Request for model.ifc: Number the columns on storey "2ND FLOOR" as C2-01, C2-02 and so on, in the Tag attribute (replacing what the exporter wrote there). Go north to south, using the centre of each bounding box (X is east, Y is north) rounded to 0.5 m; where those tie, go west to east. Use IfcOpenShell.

First a look at what the model holds.

```python
import ifcopenshell
import ifcopenshell.util.element
import ifcopenshell.util.placement

model = ifcopenshell.open("model.ifc")
print(model.schema)
storey = next(s for s in model.by_type("IfcBuildingStorey") if s.Name == "2ND FLOOR")
columns = [e for e in ifcopenshell.util.element.get_decomposition(storey) if e.is_a("IfcColumn")]
for e in sorted(columns, key=lambda e: e.id()):
    origin = ifcopenshell.util.placement.get_local_placement(e.ObjectPlacement)[:3, 3]
    print(e.id(), e.Tag, e.Name, origin.round(2) + 0.0, sep=" | ")
```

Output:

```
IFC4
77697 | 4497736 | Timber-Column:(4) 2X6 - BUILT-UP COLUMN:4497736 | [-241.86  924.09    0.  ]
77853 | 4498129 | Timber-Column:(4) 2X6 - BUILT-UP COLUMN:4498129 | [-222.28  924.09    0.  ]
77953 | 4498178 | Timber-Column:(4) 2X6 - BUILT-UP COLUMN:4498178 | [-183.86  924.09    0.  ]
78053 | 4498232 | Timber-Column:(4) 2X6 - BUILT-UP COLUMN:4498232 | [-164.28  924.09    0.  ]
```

```python
import ifcopenshell
import ifcopenshell.geom
import ifcopenshell.util.element
import ifcopenshell.util.shape

model = ifcopenshell.open("model.ifc")
settings = ifcopenshell.geom.settings()
settings.set("use-world-coords", True)


def centre(element):
    shape = ifcopenshell.geom.create_shape(settings, element)
    return ifcopenshell.util.shape.get_bbox_centroid(shape.geometry)


storey = next(s for s in model.by_type("IfcBuildingStorey") if s.Name == "2ND FLOOR")
columns = [e for e in ifcopenshell.util.element.get_decomposition(storey) if e.is_a("IfcColumn")]

# Insertion points can sit at a corner or the storey origin, so sort by the geometry (in metres).
centres = {e: centre(e) for e in columns}
columns.sort(key=lambda e: (-round(centres[e][1] / 0.5), centres[e][0]))

for i, e in enumerate(columns, start=1):
    number = f"C2-{i:02d}"
    e.Tag = number
    print(e.id(), number)

model.write("model_v2.ifc")
```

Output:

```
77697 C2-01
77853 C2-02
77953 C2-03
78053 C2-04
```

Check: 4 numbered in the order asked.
